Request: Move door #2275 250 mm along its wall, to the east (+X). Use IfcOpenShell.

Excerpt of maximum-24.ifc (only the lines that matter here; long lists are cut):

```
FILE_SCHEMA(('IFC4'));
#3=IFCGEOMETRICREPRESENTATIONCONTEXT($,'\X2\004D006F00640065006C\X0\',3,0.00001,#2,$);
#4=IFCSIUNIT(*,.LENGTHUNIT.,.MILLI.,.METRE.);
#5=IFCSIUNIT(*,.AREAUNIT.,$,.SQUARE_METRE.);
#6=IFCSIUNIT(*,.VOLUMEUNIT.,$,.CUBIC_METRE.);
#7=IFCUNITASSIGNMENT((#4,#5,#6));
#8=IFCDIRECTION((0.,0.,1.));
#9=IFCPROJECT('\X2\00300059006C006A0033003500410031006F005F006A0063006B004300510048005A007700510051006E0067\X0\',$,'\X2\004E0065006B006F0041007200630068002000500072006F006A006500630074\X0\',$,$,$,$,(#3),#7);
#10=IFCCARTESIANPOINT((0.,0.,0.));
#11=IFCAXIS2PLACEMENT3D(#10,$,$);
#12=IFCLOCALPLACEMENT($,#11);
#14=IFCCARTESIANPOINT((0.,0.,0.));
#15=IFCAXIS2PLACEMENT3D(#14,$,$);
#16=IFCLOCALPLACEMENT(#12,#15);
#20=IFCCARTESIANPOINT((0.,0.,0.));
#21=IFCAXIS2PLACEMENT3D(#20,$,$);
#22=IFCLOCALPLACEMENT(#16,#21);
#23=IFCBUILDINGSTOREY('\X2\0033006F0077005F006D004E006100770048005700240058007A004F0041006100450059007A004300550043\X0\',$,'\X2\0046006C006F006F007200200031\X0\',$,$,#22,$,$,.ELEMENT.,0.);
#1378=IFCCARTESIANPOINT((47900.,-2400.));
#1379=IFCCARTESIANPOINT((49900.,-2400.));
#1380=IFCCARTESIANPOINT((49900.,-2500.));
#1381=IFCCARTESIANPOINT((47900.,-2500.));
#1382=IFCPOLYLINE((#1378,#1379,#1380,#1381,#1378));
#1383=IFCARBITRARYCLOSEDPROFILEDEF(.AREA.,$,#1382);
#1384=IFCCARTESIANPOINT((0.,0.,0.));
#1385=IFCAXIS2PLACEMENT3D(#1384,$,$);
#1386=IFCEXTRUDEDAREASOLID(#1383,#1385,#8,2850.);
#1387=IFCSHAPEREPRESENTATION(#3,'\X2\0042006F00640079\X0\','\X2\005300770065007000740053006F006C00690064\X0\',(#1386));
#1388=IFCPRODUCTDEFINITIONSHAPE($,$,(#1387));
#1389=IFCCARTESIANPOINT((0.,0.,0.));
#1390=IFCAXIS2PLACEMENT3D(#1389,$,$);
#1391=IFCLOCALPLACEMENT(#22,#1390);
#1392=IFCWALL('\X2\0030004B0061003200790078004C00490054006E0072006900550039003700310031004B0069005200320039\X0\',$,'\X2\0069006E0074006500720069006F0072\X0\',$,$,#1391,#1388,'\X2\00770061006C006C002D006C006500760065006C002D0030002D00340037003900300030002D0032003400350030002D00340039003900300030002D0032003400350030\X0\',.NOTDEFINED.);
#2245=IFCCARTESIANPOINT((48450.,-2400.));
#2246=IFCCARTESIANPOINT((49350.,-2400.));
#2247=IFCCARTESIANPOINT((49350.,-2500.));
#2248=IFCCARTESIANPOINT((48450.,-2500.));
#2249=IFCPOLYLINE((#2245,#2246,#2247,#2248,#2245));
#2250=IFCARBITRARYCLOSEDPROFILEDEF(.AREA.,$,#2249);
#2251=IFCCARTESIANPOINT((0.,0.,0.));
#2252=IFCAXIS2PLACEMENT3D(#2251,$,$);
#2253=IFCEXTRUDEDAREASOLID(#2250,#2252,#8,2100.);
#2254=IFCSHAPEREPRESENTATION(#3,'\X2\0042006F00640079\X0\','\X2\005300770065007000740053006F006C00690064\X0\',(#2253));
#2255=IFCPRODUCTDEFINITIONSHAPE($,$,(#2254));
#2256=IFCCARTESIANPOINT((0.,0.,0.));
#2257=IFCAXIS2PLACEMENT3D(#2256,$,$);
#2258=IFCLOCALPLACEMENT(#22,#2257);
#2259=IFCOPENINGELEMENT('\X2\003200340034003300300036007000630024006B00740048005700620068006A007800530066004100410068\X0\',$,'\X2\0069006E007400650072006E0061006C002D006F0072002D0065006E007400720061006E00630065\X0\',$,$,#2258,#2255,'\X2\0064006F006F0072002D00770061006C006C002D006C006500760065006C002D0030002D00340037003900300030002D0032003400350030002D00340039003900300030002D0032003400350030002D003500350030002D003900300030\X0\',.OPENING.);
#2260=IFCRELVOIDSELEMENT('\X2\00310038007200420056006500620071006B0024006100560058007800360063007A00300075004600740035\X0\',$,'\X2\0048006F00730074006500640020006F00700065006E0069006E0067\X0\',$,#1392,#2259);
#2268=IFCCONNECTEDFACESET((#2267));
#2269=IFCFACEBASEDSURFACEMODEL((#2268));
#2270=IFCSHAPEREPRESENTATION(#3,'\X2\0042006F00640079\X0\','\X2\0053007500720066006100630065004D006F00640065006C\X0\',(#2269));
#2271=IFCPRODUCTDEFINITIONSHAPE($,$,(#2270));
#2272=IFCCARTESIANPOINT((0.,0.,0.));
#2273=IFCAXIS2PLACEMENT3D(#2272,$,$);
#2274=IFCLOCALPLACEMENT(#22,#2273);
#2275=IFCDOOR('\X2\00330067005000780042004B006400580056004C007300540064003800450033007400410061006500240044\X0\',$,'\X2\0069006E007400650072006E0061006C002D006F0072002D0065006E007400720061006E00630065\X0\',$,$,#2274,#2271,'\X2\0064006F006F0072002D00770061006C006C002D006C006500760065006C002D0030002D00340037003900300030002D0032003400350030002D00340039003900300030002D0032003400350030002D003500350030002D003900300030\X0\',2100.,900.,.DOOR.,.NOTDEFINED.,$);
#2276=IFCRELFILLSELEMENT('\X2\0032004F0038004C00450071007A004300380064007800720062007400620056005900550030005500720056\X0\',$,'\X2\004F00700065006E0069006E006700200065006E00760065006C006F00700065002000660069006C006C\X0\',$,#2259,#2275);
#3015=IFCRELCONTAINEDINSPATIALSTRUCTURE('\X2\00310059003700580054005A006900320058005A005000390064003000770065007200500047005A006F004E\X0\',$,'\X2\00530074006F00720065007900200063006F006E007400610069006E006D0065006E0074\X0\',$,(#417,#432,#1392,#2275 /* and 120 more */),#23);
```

```python
import ifcopenshell
import ifcopenshell.api.geometry
import ifcopenshell.util.placement
import ifcopenshell.util.unit

model = ifcopenshell.open("maximum-24.ifc")
unit_scale = ifcopenshell.util.unit.calculate_unit_scale(model)

door = model.by_guid("3gPxBKdXVLsTd8E3tAae$D")
opening = door.FillsVoids[0].RelatingOpeningElement
wall = opening.VoidsElements[0].RelatingBuildingElement

wall_matrix = ifcopenshell.util.placement.get_local_placement(wall.ObjectPlacement)
shift = wall_matrix[:3, 0] * 0.25 / unit_scale
before = ifcopenshell.util.placement.get_local_placement(door.ObjectPlacement)[:3, 3].copy()

# The door is not placed relative to its opening, so move both.
for product in (opening, door):
    matrix = ifcopenshell.util.placement.get_local_placement(product.ObjectPlacement)
    matrix[:3, 3] += shift
    ifcopenshell.api.geometry.edit_object_placement(model, product=product, matrix=matrix, is_si=False)

after = ifcopenshell.util.placement.get_local_placement(door.ObjectPlacement)[:3, 3]
print("door moved by", (after - before).round(3) + 0.0)

model.write("maximum-24_rev.ifc")
```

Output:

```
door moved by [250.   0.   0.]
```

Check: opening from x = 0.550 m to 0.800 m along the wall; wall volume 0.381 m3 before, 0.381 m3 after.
